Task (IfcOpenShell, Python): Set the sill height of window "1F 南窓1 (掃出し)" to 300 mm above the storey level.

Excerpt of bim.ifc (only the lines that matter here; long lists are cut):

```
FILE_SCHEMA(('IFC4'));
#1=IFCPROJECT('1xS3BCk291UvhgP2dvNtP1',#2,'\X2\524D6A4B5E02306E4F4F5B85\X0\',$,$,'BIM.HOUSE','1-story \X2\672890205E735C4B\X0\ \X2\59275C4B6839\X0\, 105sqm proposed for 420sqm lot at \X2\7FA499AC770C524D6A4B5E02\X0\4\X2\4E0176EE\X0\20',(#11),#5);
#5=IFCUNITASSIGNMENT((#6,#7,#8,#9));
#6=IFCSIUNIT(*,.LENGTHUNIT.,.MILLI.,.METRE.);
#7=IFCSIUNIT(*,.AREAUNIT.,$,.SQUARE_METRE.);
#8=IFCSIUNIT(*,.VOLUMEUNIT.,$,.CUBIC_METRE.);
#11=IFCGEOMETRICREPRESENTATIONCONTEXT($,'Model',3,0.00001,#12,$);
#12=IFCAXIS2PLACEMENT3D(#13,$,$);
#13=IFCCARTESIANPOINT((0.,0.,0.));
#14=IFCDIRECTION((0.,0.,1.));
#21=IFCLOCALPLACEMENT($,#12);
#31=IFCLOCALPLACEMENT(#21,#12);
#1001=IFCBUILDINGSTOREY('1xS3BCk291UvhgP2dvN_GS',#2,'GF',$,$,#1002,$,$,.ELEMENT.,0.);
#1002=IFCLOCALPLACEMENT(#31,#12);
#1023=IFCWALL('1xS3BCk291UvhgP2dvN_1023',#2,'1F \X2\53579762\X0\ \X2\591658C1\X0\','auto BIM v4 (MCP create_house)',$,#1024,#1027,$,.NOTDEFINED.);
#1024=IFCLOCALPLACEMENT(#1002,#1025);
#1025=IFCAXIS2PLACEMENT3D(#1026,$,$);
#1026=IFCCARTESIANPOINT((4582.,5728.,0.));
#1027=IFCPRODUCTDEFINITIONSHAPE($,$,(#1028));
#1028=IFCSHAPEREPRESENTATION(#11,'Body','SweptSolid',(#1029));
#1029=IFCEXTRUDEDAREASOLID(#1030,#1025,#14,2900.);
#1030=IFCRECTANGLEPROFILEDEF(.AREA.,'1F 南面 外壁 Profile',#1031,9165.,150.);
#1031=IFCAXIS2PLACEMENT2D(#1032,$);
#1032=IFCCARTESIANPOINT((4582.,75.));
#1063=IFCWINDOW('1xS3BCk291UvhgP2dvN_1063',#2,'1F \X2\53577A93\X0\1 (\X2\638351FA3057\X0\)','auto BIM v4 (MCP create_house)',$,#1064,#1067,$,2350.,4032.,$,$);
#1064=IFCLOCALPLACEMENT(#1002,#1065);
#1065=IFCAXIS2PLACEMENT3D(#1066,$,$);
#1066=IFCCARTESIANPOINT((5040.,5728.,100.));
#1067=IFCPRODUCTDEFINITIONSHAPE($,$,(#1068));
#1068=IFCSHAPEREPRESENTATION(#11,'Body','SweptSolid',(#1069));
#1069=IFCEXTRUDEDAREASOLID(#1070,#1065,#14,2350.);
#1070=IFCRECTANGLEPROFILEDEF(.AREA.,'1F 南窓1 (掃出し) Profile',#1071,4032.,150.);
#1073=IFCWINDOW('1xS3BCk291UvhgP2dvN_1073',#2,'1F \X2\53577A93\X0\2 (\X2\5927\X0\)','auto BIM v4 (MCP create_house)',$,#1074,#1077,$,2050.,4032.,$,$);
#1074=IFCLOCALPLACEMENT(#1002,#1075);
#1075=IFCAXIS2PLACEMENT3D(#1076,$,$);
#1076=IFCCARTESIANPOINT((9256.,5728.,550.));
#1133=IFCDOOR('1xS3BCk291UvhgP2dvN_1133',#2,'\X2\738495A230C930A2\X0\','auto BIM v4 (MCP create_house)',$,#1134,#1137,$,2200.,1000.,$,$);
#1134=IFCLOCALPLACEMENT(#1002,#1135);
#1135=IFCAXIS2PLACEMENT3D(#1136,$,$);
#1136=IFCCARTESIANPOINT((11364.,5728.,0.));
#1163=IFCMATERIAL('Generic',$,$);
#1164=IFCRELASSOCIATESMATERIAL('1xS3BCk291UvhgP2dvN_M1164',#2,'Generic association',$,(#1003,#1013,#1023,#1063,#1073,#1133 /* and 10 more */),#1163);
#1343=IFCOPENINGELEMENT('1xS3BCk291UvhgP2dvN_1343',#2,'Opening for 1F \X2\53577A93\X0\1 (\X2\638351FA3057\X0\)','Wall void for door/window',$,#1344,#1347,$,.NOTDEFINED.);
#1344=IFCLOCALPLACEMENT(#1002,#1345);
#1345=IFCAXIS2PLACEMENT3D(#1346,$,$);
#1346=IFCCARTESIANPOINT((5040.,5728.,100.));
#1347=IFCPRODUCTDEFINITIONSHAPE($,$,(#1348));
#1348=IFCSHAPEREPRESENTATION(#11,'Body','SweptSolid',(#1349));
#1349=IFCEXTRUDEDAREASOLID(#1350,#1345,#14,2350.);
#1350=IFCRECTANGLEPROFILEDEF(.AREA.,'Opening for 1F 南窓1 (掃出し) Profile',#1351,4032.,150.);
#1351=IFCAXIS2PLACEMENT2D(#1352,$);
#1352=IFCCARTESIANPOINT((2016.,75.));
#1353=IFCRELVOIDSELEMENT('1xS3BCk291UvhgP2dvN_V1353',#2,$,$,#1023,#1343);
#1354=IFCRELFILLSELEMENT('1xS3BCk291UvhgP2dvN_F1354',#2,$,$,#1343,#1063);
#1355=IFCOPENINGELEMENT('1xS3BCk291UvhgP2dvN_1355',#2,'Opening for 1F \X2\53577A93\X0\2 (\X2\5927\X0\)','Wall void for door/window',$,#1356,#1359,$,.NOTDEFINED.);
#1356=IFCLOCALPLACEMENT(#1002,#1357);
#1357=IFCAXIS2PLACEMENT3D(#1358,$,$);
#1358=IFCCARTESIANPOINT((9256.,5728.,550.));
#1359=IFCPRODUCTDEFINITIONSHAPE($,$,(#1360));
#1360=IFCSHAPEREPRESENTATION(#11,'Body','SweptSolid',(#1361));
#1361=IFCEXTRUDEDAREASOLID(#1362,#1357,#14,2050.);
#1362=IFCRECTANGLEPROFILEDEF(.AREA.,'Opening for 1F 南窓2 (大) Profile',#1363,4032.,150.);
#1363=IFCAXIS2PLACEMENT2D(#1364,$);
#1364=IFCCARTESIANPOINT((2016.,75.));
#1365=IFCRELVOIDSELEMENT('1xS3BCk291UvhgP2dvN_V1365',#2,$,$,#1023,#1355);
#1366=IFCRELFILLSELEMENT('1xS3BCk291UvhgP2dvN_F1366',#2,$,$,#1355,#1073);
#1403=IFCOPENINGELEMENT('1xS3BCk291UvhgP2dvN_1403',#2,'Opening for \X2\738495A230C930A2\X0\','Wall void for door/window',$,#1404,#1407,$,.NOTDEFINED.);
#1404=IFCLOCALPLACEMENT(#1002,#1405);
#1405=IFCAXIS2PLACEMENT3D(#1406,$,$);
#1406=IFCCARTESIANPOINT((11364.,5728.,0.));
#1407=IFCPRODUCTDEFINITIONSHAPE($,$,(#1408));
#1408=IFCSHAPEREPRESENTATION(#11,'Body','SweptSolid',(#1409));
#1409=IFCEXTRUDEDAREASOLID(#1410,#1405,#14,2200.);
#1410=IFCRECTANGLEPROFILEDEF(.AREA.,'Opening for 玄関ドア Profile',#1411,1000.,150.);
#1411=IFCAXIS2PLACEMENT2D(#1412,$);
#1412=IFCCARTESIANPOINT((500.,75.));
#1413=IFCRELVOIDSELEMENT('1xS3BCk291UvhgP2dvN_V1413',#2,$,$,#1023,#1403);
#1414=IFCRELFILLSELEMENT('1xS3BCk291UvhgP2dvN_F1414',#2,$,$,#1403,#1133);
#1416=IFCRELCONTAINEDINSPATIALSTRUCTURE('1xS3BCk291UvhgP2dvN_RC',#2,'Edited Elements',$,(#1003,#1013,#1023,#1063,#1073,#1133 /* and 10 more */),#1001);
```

```python
import numpy as np
import ifcopenshell
import ifcopenshell.api.geometry
import ifcopenshell.geom
import ifcopenshell.util.element
import ifcopenshell.util.placement
import ifcopenshell.util.shape
import ifcopenshell.util.unit

model = ifcopenshell.open("bim.ifc")
unit_scale = ifcopenshell.util.unit.calculate_unit_scale(model)

window = model.by_guid("1xS3BCk291UvhgP2dvN_1063")
opening = window.FillsVoids[0].RelatingOpeningElement
storey = ifcopenshell.util.element.get_container(window, ifc_class="IfcBuildingStorey")
level = ifcopenshell.util.placement.get_local_placement(storey.ObjectPlacement)[2, 3]

# The opening's origin need not be at the sill, so measure its lowest point.
shape = ifcopenshell.geom.create_shape(ifcopenshell.geom.settings(), opening)
bottom = ifcopenshell.util.shape.get_shape_bottom_elevation(shape, shape.geometry) / unit_scale
dz = level + 0.3 / unit_scale - bottom

shift = np.array([0.0, 0.0, dz])
# The window is not placed relative to its opening, so move both.
for product in (opening, window):
    matrix = ifcopenshell.util.placement.get_local_placement(product.ObjectPlacement)
    matrix[:3, 3] += shift
    ifcopenshell.api.geometry.edit_object_placement(model, product=product, matrix=matrix, is_si=False)

print(f"moved by {dz * unit_scale:+.3f} m")

model.write("bim_rev.ifc")
```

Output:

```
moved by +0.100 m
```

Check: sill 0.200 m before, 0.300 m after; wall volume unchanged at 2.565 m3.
